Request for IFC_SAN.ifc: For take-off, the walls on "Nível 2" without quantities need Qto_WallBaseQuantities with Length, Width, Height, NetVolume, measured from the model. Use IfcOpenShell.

First a look at what the model holds.

```python
import ifcopenshell
import ifcopenshell.util.element
import ifcopenshell.util.unit

model = ifcopenshell.open("IFC_SAN.ifc")
print(model.schema)
for unit_type in ("LENGTHUNIT", "AREAUNIT", "VOLUMEUNIT"):
    print(unit_type, ifcopenshell.util.unit.calculate_unit_scale(model, unit_type))
storey = next(s for s in model.by_type("IfcBuildingStorey") if s.Name == "Nível 2")
walls = [e for e in ifcopenshell.util.element.get_decomposition(storey) if e.is_a("IfcWall")]
for e in sorted(walls, key=lambda e: e.id()):
    print(e.id(), e.is_a(), e.Name, list(ifcopenshell.util.element.get_psets(e, qtos_only=True)), sep=" | ")
```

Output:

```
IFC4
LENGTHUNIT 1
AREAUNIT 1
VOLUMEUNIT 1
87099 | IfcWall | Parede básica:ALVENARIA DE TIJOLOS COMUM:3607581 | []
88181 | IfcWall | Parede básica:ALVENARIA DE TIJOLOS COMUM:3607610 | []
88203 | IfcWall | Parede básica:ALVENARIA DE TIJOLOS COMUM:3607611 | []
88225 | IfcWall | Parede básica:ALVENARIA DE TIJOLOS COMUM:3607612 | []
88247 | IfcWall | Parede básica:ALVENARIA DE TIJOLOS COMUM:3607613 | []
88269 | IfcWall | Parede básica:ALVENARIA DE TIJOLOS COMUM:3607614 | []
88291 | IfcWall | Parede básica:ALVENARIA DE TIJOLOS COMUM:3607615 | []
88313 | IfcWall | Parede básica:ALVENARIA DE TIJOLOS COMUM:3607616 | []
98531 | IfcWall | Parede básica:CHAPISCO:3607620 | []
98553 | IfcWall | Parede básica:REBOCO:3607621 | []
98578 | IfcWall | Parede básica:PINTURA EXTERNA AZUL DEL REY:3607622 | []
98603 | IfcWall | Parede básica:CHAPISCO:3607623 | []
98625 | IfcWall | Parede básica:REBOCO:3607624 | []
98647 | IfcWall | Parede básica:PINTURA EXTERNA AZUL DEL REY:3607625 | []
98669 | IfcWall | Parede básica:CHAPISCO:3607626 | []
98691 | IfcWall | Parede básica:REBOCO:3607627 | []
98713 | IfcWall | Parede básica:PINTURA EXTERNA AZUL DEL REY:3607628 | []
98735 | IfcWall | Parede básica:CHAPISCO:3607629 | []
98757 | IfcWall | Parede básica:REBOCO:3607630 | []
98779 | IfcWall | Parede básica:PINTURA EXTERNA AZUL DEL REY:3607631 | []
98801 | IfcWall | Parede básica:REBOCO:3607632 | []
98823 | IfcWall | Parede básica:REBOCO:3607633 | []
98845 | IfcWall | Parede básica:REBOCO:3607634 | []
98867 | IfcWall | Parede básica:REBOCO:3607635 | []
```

```python
import ifcopenshell
import ifcopenshell.api.pset
import ifcopenshell.geom
import ifcopenshell.util.element
import ifcopenshell.util.shape
import ifcopenshell.util.unit

model = ifcopenshell.open("IFC_SAN.ifc")
unit_scale = ifcopenshell.util.unit.calculate_unit_scale(model)
volume_scale = ifcopenshell.util.unit.calculate_unit_scale(model, "VOLUMEUNIT")
settings = ifcopenshell.geom.settings()

storey = next(s for s in model.by_type("IfcBuildingStorey") if s.Name == "Nível 2")
walls = [e for e in ifcopenshell.util.element.get_decomposition(storey) if e.is_a("IfcWall")]

for e in sorted(walls, key=lambda e: e.id()):
    if ifcopenshell.util.element.get_psets(e, qtos_only=True, should_inherit=False):
        continue
    # Geometry comes back in metres, in the element's own axes.
    shape = ifcopenshell.geom.create_shape(settings, e)
    values = {
        "Length": ifcopenshell.util.shape.get_x(shape.geometry) / unit_scale,
        "Width": ifcopenshell.util.shape.get_y(shape.geometry) / unit_scale,
        "Height": ifcopenshell.util.shape.get_z(shape.geometry) / unit_scale,
        "NetVolume": ifcopenshell.util.shape.get_volume(shape.geometry) / volume_scale,
    }
    qto = ifcopenshell.api.pset.add_qto(model, product=e, name="Qto_WallBaseQuantities")
    ifcopenshell.api.pset.edit_qto(model, qto=qto, properties=values)
    print(e.id(), {k: round(v, 3) for k, v in values.items()})

model.write("IFC_SAN_rev.ifc")
```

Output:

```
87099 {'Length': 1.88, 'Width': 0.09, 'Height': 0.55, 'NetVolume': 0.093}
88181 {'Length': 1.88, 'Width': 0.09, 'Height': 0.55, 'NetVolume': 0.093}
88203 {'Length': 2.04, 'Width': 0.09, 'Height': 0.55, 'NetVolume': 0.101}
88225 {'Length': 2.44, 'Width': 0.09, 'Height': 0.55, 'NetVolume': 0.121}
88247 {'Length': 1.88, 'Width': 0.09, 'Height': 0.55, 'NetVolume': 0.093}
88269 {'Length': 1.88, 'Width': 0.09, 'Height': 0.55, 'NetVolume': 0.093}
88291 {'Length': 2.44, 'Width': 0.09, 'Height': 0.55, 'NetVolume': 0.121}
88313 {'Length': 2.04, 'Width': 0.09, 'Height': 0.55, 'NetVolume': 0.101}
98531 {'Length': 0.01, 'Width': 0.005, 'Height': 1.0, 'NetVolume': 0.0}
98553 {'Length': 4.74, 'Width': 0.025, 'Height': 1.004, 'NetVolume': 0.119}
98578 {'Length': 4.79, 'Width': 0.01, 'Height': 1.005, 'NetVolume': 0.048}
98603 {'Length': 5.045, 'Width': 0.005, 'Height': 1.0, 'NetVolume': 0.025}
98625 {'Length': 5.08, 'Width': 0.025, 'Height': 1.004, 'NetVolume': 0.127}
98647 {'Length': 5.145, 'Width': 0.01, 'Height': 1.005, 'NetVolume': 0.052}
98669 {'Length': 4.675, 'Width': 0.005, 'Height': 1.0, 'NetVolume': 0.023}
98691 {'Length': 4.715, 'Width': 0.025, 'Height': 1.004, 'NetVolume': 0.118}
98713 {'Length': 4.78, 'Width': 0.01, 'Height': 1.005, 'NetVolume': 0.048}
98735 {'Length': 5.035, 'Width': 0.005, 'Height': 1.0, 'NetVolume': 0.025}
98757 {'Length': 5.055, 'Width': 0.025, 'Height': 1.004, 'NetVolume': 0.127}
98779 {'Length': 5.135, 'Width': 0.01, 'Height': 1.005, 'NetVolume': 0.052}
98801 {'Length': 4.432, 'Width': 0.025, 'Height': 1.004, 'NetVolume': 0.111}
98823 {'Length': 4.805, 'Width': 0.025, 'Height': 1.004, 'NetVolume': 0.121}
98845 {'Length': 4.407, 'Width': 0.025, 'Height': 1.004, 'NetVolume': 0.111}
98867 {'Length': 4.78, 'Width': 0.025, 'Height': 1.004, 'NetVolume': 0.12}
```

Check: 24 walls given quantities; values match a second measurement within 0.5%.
